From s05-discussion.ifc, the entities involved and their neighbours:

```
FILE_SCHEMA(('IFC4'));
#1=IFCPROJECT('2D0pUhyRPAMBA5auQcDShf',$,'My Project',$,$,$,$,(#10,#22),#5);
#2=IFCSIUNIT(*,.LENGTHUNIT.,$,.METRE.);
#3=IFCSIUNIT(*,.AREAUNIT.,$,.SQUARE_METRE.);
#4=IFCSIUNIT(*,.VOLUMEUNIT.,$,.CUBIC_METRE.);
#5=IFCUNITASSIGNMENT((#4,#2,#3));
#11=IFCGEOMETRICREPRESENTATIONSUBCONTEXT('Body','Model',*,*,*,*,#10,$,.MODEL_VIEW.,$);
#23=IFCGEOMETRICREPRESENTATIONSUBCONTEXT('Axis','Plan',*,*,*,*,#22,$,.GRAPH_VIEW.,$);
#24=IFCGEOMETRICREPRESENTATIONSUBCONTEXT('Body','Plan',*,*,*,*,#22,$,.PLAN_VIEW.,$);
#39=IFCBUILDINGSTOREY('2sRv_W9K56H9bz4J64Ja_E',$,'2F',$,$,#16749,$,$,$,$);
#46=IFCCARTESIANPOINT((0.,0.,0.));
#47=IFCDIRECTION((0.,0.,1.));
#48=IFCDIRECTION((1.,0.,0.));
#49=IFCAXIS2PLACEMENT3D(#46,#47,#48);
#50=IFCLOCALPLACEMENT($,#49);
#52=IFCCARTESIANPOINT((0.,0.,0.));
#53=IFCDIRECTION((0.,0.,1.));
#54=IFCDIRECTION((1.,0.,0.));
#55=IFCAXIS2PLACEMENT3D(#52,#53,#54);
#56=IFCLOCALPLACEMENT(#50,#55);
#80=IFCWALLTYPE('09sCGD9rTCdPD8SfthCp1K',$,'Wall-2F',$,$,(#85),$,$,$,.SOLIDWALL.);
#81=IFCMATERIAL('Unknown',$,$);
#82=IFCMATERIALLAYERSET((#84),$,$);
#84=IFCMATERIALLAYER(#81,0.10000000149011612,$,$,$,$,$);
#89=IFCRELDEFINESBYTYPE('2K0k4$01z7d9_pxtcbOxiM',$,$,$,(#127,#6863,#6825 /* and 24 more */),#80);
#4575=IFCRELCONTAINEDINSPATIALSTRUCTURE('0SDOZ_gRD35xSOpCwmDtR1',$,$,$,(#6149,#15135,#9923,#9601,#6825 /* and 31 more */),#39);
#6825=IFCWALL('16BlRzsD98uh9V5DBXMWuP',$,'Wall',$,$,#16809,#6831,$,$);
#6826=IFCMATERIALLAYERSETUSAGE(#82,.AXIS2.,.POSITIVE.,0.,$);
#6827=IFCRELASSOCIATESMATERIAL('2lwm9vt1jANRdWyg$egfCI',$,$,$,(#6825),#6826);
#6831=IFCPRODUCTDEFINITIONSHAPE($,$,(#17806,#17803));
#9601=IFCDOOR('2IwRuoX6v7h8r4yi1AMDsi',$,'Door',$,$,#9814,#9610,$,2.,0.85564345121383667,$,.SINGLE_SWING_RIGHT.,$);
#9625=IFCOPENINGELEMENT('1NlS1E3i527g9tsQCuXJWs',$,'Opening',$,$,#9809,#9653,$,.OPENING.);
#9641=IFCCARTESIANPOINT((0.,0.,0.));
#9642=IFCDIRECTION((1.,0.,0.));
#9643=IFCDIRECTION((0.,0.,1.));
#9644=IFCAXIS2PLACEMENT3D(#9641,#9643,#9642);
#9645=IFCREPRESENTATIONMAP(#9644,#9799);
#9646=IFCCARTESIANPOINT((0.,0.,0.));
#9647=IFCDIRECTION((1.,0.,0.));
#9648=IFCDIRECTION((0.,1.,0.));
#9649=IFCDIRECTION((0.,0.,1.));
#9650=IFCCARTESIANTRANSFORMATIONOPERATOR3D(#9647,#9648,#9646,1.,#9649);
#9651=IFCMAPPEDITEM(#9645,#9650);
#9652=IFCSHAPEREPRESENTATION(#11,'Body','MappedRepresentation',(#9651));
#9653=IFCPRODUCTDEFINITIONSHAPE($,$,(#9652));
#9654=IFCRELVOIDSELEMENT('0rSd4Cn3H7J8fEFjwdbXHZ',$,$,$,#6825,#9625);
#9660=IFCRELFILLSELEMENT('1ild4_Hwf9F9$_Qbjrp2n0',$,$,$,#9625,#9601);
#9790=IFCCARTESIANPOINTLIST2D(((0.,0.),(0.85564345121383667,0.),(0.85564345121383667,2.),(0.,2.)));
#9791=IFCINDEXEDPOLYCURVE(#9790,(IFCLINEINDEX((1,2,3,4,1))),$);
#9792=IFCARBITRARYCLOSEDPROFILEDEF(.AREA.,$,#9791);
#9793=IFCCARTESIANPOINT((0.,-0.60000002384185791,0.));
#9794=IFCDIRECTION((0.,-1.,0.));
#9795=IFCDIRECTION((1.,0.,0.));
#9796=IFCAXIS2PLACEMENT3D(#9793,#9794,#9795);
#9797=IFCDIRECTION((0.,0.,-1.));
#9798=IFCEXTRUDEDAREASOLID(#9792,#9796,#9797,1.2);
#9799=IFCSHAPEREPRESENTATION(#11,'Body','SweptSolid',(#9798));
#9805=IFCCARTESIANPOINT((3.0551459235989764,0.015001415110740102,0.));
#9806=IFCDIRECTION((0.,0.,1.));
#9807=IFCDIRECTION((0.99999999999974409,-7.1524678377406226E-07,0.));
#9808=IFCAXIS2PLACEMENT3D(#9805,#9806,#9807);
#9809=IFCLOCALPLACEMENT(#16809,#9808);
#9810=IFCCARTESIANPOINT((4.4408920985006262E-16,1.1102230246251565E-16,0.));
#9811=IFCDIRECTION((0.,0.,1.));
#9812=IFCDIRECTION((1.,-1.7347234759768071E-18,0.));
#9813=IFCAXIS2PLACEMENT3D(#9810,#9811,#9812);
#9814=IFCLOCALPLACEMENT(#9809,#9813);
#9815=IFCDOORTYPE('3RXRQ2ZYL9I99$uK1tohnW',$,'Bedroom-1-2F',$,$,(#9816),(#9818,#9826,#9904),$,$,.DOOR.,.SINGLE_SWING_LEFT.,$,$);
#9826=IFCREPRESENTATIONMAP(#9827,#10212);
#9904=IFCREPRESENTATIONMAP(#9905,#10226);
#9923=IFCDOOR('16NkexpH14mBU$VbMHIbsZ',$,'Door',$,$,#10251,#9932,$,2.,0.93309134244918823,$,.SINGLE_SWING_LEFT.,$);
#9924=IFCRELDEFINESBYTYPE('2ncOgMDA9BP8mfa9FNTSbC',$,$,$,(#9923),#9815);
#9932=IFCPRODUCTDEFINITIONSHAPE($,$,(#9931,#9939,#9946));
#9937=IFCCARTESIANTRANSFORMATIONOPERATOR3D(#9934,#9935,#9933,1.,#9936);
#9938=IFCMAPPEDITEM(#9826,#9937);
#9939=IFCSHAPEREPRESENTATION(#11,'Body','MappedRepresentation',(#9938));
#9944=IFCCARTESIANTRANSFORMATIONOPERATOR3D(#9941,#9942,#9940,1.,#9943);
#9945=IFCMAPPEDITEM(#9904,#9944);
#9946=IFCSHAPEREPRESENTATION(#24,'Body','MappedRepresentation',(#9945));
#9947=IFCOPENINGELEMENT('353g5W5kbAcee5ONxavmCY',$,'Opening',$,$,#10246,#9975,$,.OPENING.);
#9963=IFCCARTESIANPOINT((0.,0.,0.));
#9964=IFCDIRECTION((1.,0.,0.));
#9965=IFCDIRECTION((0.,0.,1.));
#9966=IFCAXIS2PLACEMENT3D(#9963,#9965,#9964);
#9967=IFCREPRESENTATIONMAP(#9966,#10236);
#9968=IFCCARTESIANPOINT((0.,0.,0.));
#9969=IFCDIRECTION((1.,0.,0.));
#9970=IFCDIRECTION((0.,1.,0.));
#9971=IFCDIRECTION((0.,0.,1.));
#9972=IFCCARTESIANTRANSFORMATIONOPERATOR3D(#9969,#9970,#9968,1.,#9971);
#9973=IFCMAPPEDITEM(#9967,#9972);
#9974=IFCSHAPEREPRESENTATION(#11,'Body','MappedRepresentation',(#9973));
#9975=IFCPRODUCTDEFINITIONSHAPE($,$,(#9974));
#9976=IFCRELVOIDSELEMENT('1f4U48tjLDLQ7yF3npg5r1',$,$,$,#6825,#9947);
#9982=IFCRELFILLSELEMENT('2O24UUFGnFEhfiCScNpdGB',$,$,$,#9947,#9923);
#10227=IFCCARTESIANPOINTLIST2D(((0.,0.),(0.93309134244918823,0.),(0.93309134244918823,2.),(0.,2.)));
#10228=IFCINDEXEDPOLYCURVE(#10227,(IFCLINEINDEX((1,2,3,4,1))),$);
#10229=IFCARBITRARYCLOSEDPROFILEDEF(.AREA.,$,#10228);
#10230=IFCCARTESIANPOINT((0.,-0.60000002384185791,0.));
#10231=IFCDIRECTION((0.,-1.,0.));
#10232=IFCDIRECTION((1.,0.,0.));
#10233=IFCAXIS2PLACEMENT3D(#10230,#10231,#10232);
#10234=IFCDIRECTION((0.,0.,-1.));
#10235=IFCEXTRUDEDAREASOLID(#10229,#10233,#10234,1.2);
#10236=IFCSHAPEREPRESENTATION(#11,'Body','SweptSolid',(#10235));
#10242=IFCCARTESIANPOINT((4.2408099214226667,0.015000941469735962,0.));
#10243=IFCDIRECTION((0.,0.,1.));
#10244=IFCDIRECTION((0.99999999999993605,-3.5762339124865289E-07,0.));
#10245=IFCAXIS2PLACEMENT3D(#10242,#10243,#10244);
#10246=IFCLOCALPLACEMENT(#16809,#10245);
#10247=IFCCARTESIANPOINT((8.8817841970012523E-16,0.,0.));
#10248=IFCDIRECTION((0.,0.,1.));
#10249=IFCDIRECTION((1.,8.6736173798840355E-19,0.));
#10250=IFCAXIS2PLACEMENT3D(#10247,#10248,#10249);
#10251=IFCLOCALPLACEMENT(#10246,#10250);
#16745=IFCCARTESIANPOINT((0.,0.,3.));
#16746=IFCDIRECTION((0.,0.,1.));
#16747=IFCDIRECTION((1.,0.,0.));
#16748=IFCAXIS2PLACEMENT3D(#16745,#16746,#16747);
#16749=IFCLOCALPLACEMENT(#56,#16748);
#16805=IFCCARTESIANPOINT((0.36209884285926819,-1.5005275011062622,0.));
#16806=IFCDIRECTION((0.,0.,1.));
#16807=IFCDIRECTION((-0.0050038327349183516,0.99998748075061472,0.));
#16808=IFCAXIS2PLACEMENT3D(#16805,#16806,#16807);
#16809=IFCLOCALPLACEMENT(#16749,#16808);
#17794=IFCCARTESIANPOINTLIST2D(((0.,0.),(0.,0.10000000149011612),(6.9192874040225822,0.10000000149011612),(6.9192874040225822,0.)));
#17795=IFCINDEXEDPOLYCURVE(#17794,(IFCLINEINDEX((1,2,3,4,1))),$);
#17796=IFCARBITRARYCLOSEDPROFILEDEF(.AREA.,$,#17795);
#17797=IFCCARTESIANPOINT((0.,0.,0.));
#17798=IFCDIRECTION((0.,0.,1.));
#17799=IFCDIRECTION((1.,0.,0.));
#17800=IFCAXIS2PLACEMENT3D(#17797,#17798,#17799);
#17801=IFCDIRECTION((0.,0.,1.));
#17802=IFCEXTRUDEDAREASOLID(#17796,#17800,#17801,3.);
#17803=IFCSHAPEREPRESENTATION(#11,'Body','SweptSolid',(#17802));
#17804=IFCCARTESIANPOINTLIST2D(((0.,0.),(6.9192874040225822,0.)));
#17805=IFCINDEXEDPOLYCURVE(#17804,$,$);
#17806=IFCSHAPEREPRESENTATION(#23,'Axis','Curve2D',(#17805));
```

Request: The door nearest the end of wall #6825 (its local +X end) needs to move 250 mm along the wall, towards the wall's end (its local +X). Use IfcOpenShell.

```python
import ifcopenshell
import ifcopenshell.api.geometry
import ifcopenshell.util.placement
import ifcopenshell.util.unit

model = ifcopenshell.open("s05-discussion.ifc")
unit_scale = ifcopenshell.util.unit.calculate_unit_scale(model)

door = model.by_guid("16NkexpH14mBU$VbMHIbsZ")
opening = door.FillsVoids[0].RelatingOpeningElement
wall = opening.VoidsElements[0].RelatingBuildingElement

wall_matrix = ifcopenshell.util.placement.get_local_placement(wall.ObjectPlacement)
shift = wall_matrix[:3, 0] * 0.25 / unit_scale
before = ifcopenshell.util.placement.get_local_placement(door.ObjectPlacement)[:3, 3].copy()

# The door is placed relative to its opening, so it follows when the opening moves.
matrix = ifcopenshell.util.placement.get_local_placement(opening.ObjectPlacement)
matrix[:3, 3] += shift
ifcopenshell.api.geometry.edit_object_placement(
    model, product=opening, matrix=matrix, is_si=False, should_transform_children=True
)

after = ifcopenshell.util.placement.get_local_placement(door.ObjectPlacement)[:3, 3]
print("door moved by", (after - before).round(3) + 0.0)

model.write("s05-discussion_edited.ifc")
```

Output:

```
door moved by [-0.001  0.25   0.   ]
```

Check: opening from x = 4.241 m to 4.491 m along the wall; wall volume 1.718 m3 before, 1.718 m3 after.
